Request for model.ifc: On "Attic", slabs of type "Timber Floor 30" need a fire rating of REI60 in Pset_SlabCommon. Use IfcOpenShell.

First a look at what the model holds.

```python
import ifcopenshell
import ifcopenshell.util.element

model = ifcopenshell.open("model.ifc")
print(model.schema)
storey = next(s for s in model.by_type("IfcBuildingStorey") if s.Name == "Attic")
slabs = [e for e in ifcopenshell.util.element.get_decomposition(storey) if e.is_a("IfcSlab")]
seen = {}
for e in slabs:
    element_type = ifcopenshell.util.element.get_type(e)
    key = (element_type.Name if element_type != e and element_type else None, ifcopenshell.util.element.get_pset(e, "Pset_SlabCommon", "FireRating"))
    seen[key] = seen.get(key, 0) + 1
for (name, value), count in sorted(seen.items(), key=str):
    print(count, "x", name, "|", value)
```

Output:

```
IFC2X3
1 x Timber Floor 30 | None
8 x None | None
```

```python
import ifcopenshell
import ifcopenshell.api.pset
import ifcopenshell.util.element

model = ifcopenshell.open("model.ifc")

storey = next(s for s in model.by_type("IfcBuildingStorey") if s.Name == "Attic")
slabs = [e for e in ifcopenshell.util.element.get_decomposition(storey) if e.is_a("IfcSlab")]

count = 0
for e in slabs:
    element_type = ifcopenshell.util.element.get_type(e)
    if element_type in (None, e) or element_type.Name != "Timber Floor 30":
        continue
    # add_pset returns the element's existing set when there is one.
    pset = ifcopenshell.api.pset.add_pset(model, product=e, name="Pset_SlabCommon")
    ifcopenshell.api.pset.edit_pset(model, pset=pset, properties={"FireRating": "REI60"})
    count += 1

print(count, "slabs updated")

model.write("model_rev.ifc")
```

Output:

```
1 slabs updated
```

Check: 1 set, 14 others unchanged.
